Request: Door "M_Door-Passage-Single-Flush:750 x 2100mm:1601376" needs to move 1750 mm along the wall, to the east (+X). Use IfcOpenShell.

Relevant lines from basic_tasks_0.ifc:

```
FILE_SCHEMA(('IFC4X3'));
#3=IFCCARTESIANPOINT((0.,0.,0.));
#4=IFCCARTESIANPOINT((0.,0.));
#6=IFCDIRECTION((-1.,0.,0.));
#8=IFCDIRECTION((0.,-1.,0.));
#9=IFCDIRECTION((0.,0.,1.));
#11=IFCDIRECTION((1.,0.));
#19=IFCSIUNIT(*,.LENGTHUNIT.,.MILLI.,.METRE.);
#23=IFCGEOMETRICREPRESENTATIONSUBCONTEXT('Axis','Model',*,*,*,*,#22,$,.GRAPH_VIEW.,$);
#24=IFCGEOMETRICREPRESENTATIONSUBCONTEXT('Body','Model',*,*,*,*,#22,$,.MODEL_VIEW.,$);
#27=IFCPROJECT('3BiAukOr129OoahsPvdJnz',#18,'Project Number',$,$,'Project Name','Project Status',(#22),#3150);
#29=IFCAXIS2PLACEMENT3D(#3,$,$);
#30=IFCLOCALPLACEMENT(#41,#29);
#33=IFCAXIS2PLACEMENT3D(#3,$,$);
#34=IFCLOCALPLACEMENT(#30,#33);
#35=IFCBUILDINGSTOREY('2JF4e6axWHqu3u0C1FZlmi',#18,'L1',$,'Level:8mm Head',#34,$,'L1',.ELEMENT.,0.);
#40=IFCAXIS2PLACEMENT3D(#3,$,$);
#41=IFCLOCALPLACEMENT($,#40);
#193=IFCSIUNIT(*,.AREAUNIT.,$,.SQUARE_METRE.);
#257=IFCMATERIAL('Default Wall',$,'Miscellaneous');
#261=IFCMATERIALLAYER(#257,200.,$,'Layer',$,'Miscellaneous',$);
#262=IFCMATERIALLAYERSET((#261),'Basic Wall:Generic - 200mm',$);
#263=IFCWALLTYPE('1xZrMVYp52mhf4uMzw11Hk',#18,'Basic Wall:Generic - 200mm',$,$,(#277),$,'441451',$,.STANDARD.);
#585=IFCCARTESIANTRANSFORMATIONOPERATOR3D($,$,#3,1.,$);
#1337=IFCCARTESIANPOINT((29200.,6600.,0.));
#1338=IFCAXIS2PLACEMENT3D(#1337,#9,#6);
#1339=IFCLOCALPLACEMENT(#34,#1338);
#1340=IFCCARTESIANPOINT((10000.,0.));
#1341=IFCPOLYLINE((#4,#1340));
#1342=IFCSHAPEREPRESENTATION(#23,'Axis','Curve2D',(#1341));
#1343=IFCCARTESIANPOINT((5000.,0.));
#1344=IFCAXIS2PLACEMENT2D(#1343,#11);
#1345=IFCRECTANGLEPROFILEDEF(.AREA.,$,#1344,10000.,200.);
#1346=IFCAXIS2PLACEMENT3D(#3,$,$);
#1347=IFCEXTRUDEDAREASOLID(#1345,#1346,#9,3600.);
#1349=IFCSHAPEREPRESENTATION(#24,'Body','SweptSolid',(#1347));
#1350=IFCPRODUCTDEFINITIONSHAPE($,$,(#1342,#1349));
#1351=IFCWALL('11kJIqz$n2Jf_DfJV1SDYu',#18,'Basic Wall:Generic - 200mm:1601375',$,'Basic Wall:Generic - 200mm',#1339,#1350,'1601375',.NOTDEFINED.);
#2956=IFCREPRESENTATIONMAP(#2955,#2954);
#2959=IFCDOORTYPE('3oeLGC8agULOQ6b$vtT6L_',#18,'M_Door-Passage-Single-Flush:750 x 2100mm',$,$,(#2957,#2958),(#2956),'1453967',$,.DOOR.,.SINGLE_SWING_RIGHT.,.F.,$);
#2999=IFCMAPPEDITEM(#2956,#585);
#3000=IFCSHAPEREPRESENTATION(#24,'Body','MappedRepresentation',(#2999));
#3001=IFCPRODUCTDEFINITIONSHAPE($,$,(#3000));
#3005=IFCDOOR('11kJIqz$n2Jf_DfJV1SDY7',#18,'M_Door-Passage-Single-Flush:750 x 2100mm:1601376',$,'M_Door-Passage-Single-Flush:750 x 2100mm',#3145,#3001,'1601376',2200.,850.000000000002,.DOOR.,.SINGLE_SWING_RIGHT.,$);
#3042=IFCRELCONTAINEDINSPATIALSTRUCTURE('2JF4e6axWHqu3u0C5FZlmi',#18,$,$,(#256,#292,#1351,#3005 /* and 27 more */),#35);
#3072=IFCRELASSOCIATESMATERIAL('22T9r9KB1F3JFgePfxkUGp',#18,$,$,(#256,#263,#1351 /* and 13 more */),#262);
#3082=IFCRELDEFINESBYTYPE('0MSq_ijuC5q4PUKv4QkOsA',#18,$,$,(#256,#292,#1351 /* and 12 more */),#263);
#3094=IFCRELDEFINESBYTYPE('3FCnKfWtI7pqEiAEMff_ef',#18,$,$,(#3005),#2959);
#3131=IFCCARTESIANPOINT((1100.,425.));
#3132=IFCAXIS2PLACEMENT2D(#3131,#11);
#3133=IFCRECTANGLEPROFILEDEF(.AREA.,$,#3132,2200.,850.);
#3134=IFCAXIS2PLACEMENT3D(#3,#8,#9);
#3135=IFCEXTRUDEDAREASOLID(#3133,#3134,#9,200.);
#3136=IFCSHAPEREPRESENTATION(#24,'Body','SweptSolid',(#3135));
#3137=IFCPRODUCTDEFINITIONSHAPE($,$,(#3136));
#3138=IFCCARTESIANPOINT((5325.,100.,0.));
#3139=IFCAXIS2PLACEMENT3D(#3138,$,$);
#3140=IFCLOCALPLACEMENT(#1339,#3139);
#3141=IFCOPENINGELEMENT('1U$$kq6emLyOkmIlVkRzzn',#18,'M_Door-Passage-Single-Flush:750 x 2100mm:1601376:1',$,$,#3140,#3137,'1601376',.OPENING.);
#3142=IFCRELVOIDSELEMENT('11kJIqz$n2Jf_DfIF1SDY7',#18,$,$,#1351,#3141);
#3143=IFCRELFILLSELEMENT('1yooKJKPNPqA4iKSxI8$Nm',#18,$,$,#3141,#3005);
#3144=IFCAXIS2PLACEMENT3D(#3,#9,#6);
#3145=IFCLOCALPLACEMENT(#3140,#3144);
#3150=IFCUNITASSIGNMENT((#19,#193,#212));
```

```python
import ifcopenshell
import ifcopenshell.api.geometry
import ifcopenshell.util.placement
import ifcopenshell.util.unit

model = ifcopenshell.open("basic_tasks_0.ifc")
unit_scale = ifcopenshell.util.unit.calculate_unit_scale(model)

door = model.by_guid("11kJIqz$n2Jf_DfJV1SDY7")
opening = door.FillsVoids[0].RelatingOpeningElement
wall = opening.VoidsElements[0].RelatingBuildingElement

wall_matrix = ifcopenshell.util.placement.get_local_placement(wall.ObjectPlacement)
shift = wall_matrix[:3, 0] * -1.75 / unit_scale
before = ifcopenshell.util.placement.get_local_placement(door.ObjectPlacement)[:3, 3].copy()

# The door is placed relative to its opening, so it follows when the opening moves.
matrix = ifcopenshell.util.placement.get_local_placement(opening.ObjectPlacement)
matrix[:3, 3] += shift
ifcopenshell.api.geometry.edit_object_placement(
    model, product=opening, matrix=matrix, is_si=False, should_transform_children=True
)

after = ifcopenshell.util.placement.get_local_placement(door.ObjectPlacement)[:3, 3]
print("door moved by", (after - before).round(3) + 0.0)

model.write("basic_tasks_0_v2.ifc")
```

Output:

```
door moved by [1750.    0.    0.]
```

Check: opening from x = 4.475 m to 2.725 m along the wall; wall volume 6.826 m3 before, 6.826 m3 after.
